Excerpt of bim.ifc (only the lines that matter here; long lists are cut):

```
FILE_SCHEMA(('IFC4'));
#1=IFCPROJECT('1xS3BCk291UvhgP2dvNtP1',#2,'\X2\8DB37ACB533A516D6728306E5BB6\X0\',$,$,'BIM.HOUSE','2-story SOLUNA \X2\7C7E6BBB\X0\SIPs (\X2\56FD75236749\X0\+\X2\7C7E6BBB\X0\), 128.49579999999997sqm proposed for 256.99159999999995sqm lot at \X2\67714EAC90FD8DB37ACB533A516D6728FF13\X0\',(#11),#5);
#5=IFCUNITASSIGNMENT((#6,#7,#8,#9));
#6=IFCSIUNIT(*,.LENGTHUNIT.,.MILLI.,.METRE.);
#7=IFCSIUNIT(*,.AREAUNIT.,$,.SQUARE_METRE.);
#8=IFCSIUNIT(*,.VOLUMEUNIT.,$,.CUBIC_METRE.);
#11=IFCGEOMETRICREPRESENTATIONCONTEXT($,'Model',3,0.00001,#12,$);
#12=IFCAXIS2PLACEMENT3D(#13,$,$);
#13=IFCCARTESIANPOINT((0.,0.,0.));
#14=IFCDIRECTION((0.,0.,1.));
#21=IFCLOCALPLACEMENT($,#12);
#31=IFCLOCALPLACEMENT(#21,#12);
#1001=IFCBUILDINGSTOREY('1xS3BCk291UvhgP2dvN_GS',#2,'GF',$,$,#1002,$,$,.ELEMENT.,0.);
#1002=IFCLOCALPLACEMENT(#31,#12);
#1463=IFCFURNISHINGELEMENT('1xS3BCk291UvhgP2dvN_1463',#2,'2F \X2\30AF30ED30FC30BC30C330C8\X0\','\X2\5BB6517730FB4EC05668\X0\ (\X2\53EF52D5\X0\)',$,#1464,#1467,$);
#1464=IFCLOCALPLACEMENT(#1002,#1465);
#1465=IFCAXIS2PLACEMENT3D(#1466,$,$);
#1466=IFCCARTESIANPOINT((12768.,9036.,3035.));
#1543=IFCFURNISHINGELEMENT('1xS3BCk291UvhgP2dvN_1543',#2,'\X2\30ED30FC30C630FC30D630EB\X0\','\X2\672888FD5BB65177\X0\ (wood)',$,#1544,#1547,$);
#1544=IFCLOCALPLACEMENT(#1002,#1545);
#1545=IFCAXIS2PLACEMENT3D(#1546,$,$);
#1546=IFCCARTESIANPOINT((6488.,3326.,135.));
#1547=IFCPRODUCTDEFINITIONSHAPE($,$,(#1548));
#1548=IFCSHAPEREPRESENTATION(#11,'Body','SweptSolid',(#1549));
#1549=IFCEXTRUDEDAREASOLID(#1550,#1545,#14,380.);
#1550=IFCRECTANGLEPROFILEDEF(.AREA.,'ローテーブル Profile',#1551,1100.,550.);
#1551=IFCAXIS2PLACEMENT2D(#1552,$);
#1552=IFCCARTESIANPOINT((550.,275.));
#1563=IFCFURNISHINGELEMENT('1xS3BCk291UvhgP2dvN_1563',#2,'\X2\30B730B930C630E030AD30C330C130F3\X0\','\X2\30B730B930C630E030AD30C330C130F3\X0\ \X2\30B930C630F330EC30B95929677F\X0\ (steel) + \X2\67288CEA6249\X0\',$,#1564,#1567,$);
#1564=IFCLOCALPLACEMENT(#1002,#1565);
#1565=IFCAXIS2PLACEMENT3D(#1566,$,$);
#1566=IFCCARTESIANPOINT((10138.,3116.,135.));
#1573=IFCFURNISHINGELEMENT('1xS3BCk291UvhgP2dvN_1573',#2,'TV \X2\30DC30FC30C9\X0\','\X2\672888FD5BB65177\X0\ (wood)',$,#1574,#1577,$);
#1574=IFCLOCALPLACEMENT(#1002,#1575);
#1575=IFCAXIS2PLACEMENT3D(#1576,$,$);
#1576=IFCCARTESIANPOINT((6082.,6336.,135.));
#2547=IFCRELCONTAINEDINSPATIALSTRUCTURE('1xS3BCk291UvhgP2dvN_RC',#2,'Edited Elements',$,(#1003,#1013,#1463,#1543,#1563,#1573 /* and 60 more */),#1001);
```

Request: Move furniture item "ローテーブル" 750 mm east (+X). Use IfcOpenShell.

```python
import ifcopenshell
import ifcopenshell.api.geometry
import ifcopenshell.util.placement
import ifcopenshell.util.unit

model = ifcopenshell.open("bim.ifc")
unit_scale = ifcopenshell.util.unit.calculate_unit_scale(model)

item = model.by_id(1543)
matrix = ifcopenshell.util.placement.get_local_placement(item.ObjectPlacement)
matrix[0, 3] += 0.75 / unit_scale
ifcopenshell.api.geometry.edit_object_placement(model, product=item, matrix=matrix, is_si=False)

print(ifcopenshell.util.placement.get_local_placement(item.ObjectPlacement).round(3) + 0.0)

model.write("bim-out.ifc")
```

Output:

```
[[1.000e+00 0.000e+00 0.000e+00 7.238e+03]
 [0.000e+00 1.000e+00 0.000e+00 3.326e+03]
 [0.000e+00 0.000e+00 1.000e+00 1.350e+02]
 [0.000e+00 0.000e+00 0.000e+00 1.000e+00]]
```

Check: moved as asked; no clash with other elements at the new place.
